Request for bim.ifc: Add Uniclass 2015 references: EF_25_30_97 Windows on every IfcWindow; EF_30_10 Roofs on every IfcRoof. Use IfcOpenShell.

First a look at what the model holds.

```python
import ifcopenshell

model = ifcopenshell.open("bim.ifc")
print(model.schema)
print("classifications:", [c.Name for c in model.by_type("IfcClassification")])
for ifc_class in ("IfcDoor", "IfcRoof", "IfcStair", "IfcWall", "IfcWindow"):
    print(ifc_class, len(model.by_type(ifc_class)))
```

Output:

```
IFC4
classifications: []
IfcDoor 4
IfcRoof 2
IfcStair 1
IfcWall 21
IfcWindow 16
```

```python
import ifcopenshell
import ifcopenshell.api.classification

model = ifcopenshell.open("bim.ifc")

system = ifcopenshell.api.classification.add_classification(model, classification="Uniclass 2015")

codes = {
    "IfcWindow": ("EF_25_30_97", "Windows"),
    "IfcRoof": ("EF_30_10", "Roofs"),
}
for ifc_class, (code, name) in codes.items():
    products = model.by_type(ifc_class)
    ifcopenshell.api.classification.add_reference(
        model, products=products, classification=system, identification=code, name=name
    )
    print(code, len(products))

model.write("bim_edited.ifc")
```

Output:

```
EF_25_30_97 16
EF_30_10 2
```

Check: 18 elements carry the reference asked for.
